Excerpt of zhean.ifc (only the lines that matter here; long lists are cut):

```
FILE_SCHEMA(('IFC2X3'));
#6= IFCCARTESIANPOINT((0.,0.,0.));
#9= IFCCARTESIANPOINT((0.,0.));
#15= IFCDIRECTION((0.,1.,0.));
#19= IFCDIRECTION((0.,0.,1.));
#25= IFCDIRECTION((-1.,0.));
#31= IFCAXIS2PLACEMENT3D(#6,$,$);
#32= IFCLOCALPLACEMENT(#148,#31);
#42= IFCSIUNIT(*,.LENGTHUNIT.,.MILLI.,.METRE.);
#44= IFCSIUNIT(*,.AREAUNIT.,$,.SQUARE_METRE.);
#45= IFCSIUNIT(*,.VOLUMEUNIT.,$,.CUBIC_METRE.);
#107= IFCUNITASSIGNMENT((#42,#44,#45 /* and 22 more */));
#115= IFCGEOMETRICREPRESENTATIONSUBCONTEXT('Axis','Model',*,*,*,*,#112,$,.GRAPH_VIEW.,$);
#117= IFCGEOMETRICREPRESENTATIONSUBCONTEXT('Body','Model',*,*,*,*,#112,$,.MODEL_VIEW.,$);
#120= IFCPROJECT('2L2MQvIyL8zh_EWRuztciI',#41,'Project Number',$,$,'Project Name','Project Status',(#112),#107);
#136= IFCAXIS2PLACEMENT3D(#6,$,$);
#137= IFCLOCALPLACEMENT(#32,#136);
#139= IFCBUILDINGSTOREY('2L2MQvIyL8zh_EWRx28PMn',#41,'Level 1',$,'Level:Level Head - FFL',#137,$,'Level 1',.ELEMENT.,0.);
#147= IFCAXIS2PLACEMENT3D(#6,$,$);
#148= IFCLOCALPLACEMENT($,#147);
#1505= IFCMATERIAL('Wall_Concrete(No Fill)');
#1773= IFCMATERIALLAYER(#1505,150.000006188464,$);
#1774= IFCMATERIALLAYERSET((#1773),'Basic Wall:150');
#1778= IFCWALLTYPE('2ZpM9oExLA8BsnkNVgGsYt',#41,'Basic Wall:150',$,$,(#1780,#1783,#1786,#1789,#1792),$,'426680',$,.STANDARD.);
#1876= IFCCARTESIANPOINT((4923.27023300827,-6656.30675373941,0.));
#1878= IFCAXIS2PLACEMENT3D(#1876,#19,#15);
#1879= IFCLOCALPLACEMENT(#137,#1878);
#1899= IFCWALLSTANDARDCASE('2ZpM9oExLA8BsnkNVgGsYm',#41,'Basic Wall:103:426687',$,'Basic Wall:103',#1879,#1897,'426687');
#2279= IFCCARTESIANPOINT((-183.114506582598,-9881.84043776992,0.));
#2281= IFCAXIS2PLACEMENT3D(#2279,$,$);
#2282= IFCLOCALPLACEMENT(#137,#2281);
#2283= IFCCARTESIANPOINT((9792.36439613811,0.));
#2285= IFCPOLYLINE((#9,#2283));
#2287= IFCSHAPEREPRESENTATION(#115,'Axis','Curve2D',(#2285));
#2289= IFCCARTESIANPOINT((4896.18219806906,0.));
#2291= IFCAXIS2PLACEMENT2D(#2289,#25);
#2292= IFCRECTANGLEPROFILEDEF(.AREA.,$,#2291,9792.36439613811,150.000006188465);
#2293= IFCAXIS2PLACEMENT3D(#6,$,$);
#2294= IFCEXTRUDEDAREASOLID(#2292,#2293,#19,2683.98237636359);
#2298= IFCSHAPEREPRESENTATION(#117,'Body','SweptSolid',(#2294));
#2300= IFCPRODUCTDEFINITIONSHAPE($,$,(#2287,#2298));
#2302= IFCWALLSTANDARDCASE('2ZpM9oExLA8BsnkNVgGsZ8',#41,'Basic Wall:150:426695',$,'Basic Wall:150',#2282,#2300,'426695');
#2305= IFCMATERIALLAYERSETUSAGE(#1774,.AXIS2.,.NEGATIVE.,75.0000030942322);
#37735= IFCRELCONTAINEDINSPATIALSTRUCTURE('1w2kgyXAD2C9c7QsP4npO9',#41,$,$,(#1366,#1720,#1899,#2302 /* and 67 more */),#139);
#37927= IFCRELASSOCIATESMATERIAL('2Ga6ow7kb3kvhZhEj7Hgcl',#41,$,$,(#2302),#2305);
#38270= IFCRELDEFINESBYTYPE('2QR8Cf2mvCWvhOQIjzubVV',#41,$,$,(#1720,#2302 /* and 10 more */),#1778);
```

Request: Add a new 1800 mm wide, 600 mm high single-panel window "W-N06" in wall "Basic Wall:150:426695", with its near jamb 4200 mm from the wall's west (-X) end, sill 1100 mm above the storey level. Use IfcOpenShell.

```python
import numpy as np
import ifcopenshell
import ifcopenshell.api.feature
import ifcopenshell.api.geometry
import ifcopenshell.api.root
import ifcopenshell.api.spatial
import ifcopenshell.api.type
import ifcopenshell.geom
import ifcopenshell.util.element
import ifcopenshell.util.placement
import ifcopenshell.util.representation
import ifcopenshell.util.shape
import ifcopenshell.util.unit

model = ifcopenshell.open("zhean.ifc")
unit_scale = ifcopenshell.util.unit.calculate_unit_scale(model)
settings = ifcopenshell.geom.settings()


def volume(element):
    """Net volume in cubic metres, openings subtracted."""
    shape = ifcopenshell.geom.create_shape(settings, element)
    return ifcopenshell.util.shape.get_volume(shape.geometry)


wall = model.by_id(2302)
storey = ifcopenshell.util.element.get_container(wall, ifc_class="IfcBuildingStorey")
context = ifcopenshell.util.representation.get_context(model, "Model", "Body", "MODEL_VIEW")
before = volume(wall)

width, height, from_end, sill = 1.8, 0.6, 4.2, 1.1  # metres

# The wall runs along its own X axis, and the end named is its -X end.
wall_shape = ifcopenshell.geom.create_shape(settings, wall)
x, y, z = ifcopenshell.util.shape.get_vertices(wall_shape.geometry).T
start = x.min() + from_end
face, thickness = float(y.min()), float(y.max() - y.min())
wall_matrix = ifcopenshell.util.placement.get_local_placement(wall.ObjectPlacement)
level = ifcopenshell.util.placement.get_local_placement(storey.ObjectPlacement)[2, 3]


def in_wall(x, y):
    """Placement at x, y metres in the wall's axes, at sill height."""
    matrix = wall_matrix.copy()
    matrix[:, 3] = wall_matrix @ np.array([x / unit_scale, y / unit_scale, 0.0, 1.0])
    matrix[2, 3] = level + sill / unit_scale
    return matrix


# Opening: a box that overshoots both wall faces by 50 mm.
opening = ifcopenshell.api.root.create_entity(model, ifc_class="IfcOpeningElement")
box = ifcopenshell.api.geometry.add_wall_representation(
    model, context=context, length=width, height=height, thickness=thickness + 0.1
)
ifcopenshell.api.geometry.assign_representation(model, product=opening, representation=box)
ifcopenshell.api.geometry.edit_object_placement(model, product=opening, matrix=in_wall(start, face - 0.05), is_si=False)
ifcopenshell.api.feature.add_feature(model, feature=opening, element=wall)

window = ifcopenshell.api.root.create_entity(model, ifc_class="IfcWindow", name="W-N06")
window.OverallWidth, window.OverallHeight = width / unit_scale, height / unit_scale
body = ifcopenshell.api.geometry.add_window_representation(
    model,
    context=context,
    overall_width=window.OverallWidth,
    overall_height=window.OverallHeight,
    partition_type="SINGLE_PANEL",
)
ifcopenshell.api.geometry.assign_representation(model, product=window, representation=body)
ifcopenshell.api.spatial.assign_container(model, products=[window], relating_structure=storey)
fills = ifcopenshell.api.feature.add_filling(model, opening=opening, element=window)
fills.OwnerHistory = window.OwnerHistory  # required in IFC2X3

# IFC2X3 keeps the operation on the window style.
style = ifcopenshell.api.root.create_entity(model, ifc_class="IfcWindowStyle", name="W-N06")
style.OperationType, style.ConstructionType = "SINGLE_PANEL", "NOTDEFINED"
style.ParameterTakesPrecedence = style.Sizeable = False
ifcopenshell.api.type.assign_type(model, related_objects=[window], relating_type=style)

# Centre the window in the wall's thickness.
ifcopenshell.api.geometry.edit_object_placement(model, product=window, matrix=in_wall(start, face), is_si=False)
window_shape = ifcopenshell.geom.create_shape(settings, window)
depth = ifcopenshell.util.shape.get_vertices(window_shape.geometry)[:, 1]
offset = face + thickness / 2 - (depth.min() + depth.max()) / 2
ifcopenshell.api.geometry.edit_object_placement(model, product=window, matrix=in_wall(start, offset), is_si=False)

after = volume(wall)

print(f"wall volume {before:.3f} -> {after:.3f} m3")

model.write("zhean_edited.ifc")
```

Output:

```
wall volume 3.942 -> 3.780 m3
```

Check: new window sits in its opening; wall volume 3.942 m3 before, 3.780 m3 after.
